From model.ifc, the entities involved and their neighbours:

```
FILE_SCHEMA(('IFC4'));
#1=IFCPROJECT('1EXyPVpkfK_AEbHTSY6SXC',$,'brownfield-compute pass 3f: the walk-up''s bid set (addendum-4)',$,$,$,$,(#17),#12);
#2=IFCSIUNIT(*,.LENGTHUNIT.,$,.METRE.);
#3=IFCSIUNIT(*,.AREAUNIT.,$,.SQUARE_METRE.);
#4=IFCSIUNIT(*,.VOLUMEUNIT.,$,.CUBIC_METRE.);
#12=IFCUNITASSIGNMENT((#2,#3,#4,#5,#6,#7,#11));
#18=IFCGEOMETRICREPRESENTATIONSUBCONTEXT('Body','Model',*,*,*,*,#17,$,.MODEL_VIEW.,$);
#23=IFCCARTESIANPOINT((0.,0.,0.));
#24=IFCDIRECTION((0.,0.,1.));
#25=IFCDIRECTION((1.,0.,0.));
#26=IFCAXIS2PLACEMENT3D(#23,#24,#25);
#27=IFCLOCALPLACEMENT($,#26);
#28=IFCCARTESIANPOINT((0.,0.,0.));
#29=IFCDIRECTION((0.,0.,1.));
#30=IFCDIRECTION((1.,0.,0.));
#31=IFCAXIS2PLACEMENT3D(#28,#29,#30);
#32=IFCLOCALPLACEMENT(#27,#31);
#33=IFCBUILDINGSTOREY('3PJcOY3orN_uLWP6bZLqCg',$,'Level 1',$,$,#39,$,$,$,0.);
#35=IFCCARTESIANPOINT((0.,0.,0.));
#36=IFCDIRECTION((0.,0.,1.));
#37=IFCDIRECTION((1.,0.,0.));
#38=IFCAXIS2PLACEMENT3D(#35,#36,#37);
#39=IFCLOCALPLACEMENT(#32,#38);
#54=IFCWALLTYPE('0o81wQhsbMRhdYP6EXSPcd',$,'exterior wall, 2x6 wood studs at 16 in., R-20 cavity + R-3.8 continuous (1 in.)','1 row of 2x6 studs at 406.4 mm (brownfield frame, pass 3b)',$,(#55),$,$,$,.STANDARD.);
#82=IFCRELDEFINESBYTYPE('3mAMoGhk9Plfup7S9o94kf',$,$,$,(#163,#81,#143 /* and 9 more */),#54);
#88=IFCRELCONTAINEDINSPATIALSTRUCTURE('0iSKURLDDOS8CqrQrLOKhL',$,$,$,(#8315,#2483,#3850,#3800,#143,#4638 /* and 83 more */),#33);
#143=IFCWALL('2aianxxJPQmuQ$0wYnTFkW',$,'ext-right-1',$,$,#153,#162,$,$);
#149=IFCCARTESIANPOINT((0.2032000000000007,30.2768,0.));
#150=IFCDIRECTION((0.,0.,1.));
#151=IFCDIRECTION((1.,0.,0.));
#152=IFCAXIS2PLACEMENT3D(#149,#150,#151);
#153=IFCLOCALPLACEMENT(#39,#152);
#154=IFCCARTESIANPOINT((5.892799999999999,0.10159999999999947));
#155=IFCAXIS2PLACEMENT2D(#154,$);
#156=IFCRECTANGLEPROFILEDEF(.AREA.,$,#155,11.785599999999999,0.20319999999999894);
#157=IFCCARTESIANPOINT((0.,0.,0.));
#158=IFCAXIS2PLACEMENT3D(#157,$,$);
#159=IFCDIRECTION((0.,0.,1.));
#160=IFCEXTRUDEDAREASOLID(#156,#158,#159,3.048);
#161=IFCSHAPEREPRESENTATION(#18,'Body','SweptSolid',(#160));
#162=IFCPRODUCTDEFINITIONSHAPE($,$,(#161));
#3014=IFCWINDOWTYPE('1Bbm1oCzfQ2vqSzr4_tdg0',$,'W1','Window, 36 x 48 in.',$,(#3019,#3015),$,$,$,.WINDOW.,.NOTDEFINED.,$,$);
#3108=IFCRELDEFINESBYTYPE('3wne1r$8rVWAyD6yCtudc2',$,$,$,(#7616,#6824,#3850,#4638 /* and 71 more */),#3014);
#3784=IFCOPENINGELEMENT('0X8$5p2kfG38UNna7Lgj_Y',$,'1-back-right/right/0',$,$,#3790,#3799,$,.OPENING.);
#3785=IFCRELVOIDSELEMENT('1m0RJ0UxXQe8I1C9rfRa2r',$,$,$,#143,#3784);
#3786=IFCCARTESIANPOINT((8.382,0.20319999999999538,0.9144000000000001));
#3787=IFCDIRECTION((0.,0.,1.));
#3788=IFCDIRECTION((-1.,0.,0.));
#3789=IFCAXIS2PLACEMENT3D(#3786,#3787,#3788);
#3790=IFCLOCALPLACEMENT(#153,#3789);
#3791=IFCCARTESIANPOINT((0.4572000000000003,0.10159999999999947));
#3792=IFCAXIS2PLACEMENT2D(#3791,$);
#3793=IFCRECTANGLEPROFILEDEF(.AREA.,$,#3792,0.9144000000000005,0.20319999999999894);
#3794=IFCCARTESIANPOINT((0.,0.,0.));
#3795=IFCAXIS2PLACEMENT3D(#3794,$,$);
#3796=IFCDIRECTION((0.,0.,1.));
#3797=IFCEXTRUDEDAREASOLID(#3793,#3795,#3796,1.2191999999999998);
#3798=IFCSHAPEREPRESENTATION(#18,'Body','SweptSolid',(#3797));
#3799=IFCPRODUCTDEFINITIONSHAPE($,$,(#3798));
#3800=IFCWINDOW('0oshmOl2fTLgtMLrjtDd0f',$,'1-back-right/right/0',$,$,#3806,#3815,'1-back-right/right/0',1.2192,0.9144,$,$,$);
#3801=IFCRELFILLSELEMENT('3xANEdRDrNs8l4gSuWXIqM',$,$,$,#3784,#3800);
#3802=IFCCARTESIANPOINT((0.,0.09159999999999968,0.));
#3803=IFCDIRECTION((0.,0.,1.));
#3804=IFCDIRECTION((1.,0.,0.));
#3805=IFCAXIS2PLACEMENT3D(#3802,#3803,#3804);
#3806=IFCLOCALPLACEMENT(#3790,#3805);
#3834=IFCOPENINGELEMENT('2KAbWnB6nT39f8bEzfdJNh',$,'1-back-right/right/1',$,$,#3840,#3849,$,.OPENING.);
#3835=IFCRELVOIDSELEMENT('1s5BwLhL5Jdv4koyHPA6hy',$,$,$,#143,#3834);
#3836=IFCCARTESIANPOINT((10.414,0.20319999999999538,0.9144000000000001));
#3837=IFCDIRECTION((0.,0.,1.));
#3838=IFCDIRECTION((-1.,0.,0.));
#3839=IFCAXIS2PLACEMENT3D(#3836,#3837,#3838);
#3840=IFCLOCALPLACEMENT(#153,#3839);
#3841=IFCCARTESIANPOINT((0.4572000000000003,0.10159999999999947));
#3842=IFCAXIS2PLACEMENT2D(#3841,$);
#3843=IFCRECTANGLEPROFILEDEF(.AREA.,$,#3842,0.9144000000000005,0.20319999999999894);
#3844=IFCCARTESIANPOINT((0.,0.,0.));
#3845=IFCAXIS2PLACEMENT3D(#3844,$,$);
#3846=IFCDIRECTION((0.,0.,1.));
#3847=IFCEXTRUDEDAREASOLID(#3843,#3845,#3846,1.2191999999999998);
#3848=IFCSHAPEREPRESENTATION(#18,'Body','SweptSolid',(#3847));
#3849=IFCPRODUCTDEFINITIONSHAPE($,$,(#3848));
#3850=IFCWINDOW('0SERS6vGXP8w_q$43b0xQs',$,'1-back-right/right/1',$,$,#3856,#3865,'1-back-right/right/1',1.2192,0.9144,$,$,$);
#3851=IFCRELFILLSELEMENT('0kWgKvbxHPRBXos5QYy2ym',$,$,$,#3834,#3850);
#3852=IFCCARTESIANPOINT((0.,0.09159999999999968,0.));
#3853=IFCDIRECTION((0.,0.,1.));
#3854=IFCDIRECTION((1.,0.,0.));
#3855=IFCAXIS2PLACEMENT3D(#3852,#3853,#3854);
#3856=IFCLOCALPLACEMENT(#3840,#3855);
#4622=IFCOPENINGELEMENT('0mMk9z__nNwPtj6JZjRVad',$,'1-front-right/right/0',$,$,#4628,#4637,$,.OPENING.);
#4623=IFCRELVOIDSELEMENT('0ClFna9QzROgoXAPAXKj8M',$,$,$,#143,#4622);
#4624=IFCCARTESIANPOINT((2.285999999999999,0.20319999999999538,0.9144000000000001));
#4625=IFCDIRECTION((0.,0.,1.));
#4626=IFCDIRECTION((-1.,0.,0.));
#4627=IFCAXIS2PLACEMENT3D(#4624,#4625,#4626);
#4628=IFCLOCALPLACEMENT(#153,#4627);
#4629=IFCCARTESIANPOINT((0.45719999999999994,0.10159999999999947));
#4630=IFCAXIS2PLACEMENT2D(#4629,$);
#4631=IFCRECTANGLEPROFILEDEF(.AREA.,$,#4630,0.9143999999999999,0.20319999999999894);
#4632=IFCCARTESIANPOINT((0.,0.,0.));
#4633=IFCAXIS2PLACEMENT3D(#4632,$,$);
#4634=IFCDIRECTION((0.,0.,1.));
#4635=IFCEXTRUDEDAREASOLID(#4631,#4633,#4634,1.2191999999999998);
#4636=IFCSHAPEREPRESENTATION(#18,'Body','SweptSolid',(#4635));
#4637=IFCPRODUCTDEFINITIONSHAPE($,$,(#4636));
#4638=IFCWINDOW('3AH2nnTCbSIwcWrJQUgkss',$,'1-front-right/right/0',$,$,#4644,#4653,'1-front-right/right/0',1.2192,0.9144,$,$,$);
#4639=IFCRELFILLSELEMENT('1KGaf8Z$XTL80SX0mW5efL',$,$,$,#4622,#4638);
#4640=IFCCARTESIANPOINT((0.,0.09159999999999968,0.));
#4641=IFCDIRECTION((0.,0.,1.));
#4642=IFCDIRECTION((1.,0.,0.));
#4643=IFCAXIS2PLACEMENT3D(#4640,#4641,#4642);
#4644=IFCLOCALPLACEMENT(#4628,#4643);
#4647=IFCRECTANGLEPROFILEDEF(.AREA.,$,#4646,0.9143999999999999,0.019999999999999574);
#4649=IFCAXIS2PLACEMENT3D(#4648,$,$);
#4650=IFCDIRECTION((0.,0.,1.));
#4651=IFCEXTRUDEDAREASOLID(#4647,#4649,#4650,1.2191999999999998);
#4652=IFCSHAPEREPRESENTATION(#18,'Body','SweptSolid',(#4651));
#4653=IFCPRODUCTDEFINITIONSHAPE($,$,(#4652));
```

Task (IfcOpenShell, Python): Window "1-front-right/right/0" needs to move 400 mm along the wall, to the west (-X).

```python
import ifcopenshell
import ifcopenshell.api.geometry
import ifcopenshell.util.placement
import ifcopenshell.util.unit

model = ifcopenshell.open("model.ifc")
unit_scale = ifcopenshell.util.unit.calculate_unit_scale(model)

window = model.by_id(4638)
opening = window.FillsVoids[0].RelatingOpeningElement
wall = opening.VoidsElements[0].RelatingBuildingElement

wall_matrix = ifcopenshell.util.placement.get_local_placement(wall.ObjectPlacement)
shift = wall_matrix[:3, 0] * -0.4 / unit_scale
before = ifcopenshell.util.placement.get_local_placement(window.ObjectPlacement)[:3, 3].copy()

# The window is placed relative to its opening, so it follows when the opening moves.
matrix = ifcopenshell.util.placement.get_local_placement(opening.ObjectPlacement)
matrix[:3, 3] += shift
ifcopenshell.api.geometry.edit_object_placement(
    model, product=opening, matrix=matrix, is_si=False, should_transform_children=True
)

after = ifcopenshell.util.placement.get_local_placement(window.ObjectPlacement)[:3, 3]
print("window moved by", (after - before).round(3) + 0.0)

model.write("model_v2.ifc")
```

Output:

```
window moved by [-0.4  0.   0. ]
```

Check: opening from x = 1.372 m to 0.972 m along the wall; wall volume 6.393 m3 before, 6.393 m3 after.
